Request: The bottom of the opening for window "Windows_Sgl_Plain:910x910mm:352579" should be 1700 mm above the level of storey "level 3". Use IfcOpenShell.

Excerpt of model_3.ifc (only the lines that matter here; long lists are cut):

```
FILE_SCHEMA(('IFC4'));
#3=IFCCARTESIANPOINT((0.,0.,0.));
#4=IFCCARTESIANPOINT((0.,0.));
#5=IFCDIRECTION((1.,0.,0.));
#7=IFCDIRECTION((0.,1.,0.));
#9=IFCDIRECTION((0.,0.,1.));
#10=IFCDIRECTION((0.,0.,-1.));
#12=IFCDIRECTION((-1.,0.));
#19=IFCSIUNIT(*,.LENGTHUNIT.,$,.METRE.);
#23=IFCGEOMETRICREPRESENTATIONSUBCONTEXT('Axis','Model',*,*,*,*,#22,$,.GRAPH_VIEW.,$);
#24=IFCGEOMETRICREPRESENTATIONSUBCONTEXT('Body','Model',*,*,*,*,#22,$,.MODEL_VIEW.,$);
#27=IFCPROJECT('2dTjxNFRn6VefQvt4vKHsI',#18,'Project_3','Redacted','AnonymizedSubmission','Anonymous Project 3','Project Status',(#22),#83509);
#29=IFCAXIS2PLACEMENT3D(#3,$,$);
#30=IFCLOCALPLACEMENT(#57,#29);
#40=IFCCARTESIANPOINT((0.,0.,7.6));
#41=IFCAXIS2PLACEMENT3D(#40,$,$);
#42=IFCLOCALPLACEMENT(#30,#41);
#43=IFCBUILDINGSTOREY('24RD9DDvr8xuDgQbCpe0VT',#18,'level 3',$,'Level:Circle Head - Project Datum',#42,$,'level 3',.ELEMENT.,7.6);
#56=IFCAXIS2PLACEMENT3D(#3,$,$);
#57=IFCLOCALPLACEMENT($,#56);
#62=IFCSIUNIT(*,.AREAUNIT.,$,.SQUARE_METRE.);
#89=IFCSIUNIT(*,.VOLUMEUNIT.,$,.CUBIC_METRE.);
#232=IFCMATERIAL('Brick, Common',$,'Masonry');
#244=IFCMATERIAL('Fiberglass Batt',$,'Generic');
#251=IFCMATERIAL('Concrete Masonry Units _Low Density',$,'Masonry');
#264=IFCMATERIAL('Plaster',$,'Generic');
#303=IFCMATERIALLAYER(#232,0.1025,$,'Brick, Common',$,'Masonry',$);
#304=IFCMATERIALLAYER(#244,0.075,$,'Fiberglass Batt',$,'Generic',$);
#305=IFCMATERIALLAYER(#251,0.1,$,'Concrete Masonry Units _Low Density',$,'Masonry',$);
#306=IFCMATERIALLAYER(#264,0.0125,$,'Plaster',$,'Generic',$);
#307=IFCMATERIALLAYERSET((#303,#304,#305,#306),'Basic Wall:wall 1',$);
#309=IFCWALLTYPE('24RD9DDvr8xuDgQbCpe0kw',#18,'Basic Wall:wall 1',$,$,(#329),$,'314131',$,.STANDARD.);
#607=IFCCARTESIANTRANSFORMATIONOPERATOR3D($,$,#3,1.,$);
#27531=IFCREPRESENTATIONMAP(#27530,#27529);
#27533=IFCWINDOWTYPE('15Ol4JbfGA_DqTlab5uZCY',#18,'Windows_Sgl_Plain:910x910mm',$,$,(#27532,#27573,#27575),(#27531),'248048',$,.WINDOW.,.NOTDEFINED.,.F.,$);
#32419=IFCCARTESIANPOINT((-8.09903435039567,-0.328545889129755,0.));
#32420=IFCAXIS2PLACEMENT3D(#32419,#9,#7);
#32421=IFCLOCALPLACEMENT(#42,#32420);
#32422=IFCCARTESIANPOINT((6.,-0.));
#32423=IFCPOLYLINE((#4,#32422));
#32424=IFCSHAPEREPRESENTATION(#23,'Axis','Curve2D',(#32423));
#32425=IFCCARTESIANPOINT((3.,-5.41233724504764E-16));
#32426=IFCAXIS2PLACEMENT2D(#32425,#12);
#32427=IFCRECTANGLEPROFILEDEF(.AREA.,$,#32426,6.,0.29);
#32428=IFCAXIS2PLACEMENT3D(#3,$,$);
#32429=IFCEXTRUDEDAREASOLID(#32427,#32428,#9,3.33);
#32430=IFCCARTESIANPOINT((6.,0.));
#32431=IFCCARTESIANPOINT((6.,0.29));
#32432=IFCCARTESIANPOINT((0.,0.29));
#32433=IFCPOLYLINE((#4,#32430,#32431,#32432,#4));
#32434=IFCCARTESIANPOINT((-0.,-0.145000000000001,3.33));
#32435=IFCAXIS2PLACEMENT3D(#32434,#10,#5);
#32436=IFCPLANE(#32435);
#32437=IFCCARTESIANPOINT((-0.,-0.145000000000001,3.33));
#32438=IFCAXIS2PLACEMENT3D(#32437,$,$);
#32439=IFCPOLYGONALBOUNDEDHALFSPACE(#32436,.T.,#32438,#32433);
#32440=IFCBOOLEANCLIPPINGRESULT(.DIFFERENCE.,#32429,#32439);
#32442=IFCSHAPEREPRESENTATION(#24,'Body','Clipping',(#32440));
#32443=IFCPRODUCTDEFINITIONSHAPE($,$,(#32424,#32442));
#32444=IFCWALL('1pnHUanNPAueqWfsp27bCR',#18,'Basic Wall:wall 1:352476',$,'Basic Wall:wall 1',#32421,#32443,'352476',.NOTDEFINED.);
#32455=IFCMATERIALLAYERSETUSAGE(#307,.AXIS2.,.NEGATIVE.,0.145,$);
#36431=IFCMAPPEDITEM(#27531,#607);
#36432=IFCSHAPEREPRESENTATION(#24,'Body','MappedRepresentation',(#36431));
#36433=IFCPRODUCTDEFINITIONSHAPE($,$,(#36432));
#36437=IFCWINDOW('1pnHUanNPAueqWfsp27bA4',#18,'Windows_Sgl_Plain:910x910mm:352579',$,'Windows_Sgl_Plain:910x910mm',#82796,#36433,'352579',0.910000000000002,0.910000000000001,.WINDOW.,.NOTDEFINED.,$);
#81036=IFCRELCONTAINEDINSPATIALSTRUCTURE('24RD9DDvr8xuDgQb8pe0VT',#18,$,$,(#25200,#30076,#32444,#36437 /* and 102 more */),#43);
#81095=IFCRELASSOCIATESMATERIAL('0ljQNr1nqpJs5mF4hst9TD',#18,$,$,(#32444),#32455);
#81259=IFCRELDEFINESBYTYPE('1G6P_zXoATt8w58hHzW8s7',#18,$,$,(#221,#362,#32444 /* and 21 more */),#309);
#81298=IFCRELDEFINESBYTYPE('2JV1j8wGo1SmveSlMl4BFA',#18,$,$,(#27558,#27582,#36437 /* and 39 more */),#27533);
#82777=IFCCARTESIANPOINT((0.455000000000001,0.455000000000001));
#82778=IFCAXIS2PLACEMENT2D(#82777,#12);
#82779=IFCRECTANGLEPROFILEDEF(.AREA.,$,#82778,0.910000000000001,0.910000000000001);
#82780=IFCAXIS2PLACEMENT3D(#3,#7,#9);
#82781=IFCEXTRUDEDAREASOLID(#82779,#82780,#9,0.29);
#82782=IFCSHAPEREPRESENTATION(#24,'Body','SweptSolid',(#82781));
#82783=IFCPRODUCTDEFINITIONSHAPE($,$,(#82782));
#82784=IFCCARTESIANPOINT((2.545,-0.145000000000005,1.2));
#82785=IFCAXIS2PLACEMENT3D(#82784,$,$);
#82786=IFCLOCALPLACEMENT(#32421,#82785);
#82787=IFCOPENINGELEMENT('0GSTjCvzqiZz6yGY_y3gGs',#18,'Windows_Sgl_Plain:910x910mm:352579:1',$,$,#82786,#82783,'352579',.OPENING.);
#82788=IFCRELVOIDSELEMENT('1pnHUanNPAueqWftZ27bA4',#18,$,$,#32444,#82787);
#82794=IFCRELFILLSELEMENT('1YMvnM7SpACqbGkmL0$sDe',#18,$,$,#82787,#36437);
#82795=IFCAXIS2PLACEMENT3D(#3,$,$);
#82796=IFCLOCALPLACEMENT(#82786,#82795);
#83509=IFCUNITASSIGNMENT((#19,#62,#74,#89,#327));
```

```python
import numpy as np
import ifcopenshell
import ifcopenshell.api.geometry
import ifcopenshell.geom
import ifcopenshell.util.element
import ifcopenshell.util.placement
import ifcopenshell.util.shape
import ifcopenshell.util.unit

model = ifcopenshell.open("model_3.ifc")
unit_scale = ifcopenshell.util.unit.calculate_unit_scale(model)

window = model.by_id(36437)
opening = window.FillsVoids[0].RelatingOpeningElement
storey = ifcopenshell.util.element.get_container(window, ifc_class="IfcBuildingStorey")
level = ifcopenshell.util.placement.get_local_placement(storey.ObjectPlacement)[2, 3]

# The opening's origin need not be at the sill, so measure its lowest point.
shape = ifcopenshell.geom.create_shape(ifcopenshell.geom.settings(), opening)
bottom = ifcopenshell.util.shape.get_shape_bottom_elevation(shape, shape.geometry) / unit_scale
dz = level + 1.7 - bottom

shift = np.array([0.0, 0.0, dz])
# The window is placed relative to its opening, so it follows when the opening moves.
matrix = ifcopenshell.util.placement.get_local_placement(opening.ObjectPlacement)
matrix[:3, 3] += shift
ifcopenshell.api.geometry.edit_object_placement(
    model, product=opening, matrix=matrix, is_si=False, should_transform_children=True
)

print(f"moved by {dz * unit_scale:+.3f} m")

model.write("model_3_v2.ifc")
```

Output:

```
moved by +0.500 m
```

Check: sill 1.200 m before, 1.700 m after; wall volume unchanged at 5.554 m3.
